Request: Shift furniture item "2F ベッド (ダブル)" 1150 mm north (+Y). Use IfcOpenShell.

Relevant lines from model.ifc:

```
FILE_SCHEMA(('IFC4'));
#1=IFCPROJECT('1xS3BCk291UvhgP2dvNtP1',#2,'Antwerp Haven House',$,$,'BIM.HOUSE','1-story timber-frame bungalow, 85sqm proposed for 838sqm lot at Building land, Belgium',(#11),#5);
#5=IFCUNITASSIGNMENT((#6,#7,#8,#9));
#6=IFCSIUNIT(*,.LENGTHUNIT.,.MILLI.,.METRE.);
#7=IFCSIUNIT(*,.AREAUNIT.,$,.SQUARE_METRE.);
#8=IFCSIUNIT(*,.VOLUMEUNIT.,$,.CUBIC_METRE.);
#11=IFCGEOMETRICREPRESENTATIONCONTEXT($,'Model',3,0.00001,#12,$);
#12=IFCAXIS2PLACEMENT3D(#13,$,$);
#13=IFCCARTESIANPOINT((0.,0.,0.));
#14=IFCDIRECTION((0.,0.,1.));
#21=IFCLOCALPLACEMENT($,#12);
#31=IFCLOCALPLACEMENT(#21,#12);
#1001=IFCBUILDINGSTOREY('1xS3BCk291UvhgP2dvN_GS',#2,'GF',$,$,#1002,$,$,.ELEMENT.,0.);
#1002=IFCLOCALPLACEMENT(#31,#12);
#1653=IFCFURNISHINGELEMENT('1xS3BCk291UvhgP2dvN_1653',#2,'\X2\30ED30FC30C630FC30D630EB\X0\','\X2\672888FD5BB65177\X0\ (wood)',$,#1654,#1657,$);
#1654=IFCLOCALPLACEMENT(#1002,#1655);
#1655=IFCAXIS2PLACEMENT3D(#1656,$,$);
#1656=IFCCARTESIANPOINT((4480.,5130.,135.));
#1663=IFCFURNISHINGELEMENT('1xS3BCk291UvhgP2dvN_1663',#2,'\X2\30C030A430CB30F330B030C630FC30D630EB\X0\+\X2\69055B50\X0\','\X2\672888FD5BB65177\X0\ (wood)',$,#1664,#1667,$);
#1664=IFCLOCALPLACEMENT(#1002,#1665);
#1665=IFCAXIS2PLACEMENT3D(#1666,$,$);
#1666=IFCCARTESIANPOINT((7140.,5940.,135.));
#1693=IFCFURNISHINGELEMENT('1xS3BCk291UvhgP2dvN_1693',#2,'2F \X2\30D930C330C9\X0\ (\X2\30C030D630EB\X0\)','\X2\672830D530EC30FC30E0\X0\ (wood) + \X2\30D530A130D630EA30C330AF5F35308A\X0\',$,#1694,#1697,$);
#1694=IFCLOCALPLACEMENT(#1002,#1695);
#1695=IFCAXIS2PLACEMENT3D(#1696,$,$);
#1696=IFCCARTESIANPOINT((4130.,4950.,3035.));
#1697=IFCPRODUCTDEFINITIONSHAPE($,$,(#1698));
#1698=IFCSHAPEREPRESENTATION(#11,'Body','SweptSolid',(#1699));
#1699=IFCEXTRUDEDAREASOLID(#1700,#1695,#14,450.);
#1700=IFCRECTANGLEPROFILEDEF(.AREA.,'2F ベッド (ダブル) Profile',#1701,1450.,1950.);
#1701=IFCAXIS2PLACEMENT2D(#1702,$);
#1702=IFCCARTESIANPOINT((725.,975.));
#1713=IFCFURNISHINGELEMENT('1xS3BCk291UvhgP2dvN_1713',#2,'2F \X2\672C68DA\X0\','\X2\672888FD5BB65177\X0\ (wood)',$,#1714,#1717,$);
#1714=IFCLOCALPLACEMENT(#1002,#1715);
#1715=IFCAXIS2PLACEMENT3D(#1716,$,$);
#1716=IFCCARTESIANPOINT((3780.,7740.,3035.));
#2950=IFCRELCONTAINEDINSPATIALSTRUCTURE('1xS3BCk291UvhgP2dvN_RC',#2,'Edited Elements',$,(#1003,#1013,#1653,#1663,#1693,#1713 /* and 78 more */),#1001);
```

```python
import ifcopenshell
import ifcopenshell.api.geometry
import ifcopenshell.util.placement

model = ifcopenshell.open("model.ifc")

item = model.by_id(1693)
matrix = ifcopenshell.util.placement.get_local_placement(item.ObjectPlacement)
matrix[1, 3] += 1150.0
ifcopenshell.api.geometry.edit_object_placement(model, product=item, matrix=matrix, is_si=False)

print(ifcopenshell.util.placement.get_local_placement(item.ObjectPlacement).round(3) + 0.0)

model.write("model_edited.ifc")
```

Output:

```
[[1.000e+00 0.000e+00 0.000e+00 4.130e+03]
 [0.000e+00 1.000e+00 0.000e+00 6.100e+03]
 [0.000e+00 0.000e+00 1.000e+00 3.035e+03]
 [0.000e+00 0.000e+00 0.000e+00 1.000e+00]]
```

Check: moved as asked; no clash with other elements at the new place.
